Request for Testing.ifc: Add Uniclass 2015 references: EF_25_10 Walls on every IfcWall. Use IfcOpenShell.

First a look at what the model holds.

```python
import ifcopenshell

model = ifcopenshell.open("Testing.ifc")
print(model.schema)
print("classifications:", [c.Name for c in model.by_type("IfcClassification")])
for ifc_class in ("IfcDoor", "IfcRoof", "IfcStair", "IfcWall", "IfcWindow"):
    print(ifc_class, len(model.by_type(ifc_class)))
```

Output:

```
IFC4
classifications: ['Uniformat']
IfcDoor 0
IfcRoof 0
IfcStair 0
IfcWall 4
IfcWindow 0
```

```python
import ifcopenshell
import ifcopenshell.api.classification

model = ifcopenshell.open("Testing.ifc")

system = ifcopenshell.api.classification.add_classification(model, classification="Uniclass 2015")

codes = {
    "IfcWall": ("EF_25_10", "Walls"),
}
for ifc_class, (code, name) in codes.items():
    products = model.by_type(ifc_class)
    ifcopenshell.api.classification.add_reference(
        model, products=products, classification=system, identification=code, name=name
    )
    print(code, len(products))

model.write("Testing_v2.ifc")
```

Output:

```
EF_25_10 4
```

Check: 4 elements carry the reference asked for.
